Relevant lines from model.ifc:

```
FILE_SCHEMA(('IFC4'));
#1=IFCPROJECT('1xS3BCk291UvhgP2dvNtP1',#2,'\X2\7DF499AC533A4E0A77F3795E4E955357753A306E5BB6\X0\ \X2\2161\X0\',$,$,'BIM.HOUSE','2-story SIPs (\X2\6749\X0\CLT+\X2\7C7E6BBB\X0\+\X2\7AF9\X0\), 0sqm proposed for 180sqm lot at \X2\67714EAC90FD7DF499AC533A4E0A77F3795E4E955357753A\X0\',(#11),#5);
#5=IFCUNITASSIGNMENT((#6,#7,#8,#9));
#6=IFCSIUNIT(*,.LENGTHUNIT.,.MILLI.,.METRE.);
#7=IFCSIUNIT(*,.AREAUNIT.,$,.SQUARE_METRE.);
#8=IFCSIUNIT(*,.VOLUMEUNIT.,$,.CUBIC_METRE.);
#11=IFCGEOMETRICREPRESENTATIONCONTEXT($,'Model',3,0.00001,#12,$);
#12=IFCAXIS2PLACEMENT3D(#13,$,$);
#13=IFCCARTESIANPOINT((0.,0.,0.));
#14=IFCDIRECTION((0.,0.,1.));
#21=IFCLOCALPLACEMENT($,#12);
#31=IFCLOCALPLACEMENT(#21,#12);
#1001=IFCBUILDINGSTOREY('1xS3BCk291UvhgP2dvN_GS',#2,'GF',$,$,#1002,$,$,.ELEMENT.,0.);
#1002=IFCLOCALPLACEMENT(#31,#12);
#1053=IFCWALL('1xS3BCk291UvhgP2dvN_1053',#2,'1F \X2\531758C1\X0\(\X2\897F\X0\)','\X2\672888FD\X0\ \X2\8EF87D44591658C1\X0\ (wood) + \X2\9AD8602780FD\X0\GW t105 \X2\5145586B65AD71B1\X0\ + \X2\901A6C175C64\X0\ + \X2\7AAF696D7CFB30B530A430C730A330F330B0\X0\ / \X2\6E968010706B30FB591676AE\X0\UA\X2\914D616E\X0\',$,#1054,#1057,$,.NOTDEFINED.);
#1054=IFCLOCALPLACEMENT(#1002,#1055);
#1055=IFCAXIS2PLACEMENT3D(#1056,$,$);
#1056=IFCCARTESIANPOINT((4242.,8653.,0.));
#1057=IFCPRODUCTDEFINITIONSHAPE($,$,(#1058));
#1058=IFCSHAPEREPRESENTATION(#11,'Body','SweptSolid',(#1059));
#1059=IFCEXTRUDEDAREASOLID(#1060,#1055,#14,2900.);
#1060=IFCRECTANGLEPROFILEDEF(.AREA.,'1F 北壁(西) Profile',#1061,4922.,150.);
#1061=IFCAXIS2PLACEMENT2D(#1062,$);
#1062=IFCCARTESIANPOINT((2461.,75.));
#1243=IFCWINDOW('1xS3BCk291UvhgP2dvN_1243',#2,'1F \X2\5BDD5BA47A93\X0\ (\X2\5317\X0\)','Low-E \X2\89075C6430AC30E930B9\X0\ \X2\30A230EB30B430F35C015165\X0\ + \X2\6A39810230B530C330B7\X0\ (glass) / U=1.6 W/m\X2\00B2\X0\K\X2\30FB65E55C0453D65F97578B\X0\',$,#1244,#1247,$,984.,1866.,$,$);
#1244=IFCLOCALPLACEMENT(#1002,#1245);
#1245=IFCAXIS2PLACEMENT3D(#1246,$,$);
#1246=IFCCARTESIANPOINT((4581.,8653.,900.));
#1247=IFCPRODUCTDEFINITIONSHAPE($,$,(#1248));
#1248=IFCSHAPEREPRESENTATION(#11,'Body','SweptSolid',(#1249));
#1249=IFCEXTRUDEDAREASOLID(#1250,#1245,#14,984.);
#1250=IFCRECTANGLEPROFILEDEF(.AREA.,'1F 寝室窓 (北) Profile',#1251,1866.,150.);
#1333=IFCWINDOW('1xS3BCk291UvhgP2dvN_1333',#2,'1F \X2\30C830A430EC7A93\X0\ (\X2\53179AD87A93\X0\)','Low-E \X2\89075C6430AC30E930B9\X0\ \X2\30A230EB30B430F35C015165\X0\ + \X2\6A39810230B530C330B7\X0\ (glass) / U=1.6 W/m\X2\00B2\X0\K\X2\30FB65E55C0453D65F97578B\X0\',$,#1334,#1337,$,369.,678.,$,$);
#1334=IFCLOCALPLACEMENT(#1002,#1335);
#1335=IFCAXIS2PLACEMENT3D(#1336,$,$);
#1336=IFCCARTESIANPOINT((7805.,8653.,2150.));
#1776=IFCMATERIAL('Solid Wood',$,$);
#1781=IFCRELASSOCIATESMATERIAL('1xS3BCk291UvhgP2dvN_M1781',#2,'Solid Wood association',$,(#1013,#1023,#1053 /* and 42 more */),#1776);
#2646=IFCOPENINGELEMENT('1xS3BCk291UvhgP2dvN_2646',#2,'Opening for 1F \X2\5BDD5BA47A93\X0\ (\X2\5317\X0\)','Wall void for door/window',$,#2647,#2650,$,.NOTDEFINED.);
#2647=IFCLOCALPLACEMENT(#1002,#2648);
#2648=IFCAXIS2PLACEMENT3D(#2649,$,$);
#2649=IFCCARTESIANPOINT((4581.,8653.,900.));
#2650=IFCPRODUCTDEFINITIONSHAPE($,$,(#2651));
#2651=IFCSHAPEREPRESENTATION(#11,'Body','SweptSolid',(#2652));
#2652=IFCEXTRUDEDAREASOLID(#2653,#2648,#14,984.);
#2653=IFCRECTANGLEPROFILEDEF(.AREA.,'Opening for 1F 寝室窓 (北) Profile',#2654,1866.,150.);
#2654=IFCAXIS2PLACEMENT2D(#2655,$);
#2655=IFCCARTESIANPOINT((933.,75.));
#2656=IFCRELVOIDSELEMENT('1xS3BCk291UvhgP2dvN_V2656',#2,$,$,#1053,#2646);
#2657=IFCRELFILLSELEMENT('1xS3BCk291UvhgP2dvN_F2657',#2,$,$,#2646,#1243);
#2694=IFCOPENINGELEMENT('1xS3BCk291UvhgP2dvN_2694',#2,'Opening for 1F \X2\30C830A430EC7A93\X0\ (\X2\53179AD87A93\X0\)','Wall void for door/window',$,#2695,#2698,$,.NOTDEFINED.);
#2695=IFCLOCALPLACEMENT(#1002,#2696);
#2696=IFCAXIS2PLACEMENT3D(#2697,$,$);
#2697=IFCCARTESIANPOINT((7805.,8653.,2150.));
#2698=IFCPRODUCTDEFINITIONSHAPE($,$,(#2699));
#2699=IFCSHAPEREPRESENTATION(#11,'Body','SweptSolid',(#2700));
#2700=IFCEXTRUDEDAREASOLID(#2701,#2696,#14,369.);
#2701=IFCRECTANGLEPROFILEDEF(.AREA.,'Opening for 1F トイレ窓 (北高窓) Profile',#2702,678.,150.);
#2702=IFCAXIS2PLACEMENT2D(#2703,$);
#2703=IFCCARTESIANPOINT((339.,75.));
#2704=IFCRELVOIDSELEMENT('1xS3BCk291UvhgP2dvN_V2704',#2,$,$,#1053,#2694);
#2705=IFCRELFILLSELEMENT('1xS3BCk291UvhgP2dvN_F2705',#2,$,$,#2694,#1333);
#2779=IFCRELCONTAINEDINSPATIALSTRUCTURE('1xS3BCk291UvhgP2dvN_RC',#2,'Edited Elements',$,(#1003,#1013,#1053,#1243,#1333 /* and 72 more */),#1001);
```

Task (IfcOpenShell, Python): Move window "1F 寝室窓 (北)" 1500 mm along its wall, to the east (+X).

```python
import ifcopenshell
import ifcopenshell.api.geometry
import ifcopenshell.util.placement

model = ifcopenshell.open("model.ifc")

window = model.by_guid("1xS3BCk291UvhgP2dvN_1243")
opening = window.FillsVoids[0].RelatingOpeningElement
wall = opening.VoidsElements[0].RelatingBuildingElement

wall_matrix = ifcopenshell.util.placement.get_local_placement(wall.ObjectPlacement)
shift = wall_matrix[:3, 0] * 1500.0
before = ifcopenshell.util.placement.get_local_placement(window.ObjectPlacement)[:3, 3].copy()

# The window is not placed relative to its opening, so move both.
for product in (opening, window):
    matrix = ifcopenshell.util.placement.get_local_placement(product.ObjectPlacement)
    matrix[:3, 3] += shift
    ifcopenshell.api.geometry.edit_object_placement(model, product=product, matrix=matrix, is_si=False)

after = ifcopenshell.util.placement.get_local_placement(window.ObjectPlacement)[:3, 3]
print("window moved by", (after - before).round(3) + 0.0)

model.write("model_rev.ifc")
```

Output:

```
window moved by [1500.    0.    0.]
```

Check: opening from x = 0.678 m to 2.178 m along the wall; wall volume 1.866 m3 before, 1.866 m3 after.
